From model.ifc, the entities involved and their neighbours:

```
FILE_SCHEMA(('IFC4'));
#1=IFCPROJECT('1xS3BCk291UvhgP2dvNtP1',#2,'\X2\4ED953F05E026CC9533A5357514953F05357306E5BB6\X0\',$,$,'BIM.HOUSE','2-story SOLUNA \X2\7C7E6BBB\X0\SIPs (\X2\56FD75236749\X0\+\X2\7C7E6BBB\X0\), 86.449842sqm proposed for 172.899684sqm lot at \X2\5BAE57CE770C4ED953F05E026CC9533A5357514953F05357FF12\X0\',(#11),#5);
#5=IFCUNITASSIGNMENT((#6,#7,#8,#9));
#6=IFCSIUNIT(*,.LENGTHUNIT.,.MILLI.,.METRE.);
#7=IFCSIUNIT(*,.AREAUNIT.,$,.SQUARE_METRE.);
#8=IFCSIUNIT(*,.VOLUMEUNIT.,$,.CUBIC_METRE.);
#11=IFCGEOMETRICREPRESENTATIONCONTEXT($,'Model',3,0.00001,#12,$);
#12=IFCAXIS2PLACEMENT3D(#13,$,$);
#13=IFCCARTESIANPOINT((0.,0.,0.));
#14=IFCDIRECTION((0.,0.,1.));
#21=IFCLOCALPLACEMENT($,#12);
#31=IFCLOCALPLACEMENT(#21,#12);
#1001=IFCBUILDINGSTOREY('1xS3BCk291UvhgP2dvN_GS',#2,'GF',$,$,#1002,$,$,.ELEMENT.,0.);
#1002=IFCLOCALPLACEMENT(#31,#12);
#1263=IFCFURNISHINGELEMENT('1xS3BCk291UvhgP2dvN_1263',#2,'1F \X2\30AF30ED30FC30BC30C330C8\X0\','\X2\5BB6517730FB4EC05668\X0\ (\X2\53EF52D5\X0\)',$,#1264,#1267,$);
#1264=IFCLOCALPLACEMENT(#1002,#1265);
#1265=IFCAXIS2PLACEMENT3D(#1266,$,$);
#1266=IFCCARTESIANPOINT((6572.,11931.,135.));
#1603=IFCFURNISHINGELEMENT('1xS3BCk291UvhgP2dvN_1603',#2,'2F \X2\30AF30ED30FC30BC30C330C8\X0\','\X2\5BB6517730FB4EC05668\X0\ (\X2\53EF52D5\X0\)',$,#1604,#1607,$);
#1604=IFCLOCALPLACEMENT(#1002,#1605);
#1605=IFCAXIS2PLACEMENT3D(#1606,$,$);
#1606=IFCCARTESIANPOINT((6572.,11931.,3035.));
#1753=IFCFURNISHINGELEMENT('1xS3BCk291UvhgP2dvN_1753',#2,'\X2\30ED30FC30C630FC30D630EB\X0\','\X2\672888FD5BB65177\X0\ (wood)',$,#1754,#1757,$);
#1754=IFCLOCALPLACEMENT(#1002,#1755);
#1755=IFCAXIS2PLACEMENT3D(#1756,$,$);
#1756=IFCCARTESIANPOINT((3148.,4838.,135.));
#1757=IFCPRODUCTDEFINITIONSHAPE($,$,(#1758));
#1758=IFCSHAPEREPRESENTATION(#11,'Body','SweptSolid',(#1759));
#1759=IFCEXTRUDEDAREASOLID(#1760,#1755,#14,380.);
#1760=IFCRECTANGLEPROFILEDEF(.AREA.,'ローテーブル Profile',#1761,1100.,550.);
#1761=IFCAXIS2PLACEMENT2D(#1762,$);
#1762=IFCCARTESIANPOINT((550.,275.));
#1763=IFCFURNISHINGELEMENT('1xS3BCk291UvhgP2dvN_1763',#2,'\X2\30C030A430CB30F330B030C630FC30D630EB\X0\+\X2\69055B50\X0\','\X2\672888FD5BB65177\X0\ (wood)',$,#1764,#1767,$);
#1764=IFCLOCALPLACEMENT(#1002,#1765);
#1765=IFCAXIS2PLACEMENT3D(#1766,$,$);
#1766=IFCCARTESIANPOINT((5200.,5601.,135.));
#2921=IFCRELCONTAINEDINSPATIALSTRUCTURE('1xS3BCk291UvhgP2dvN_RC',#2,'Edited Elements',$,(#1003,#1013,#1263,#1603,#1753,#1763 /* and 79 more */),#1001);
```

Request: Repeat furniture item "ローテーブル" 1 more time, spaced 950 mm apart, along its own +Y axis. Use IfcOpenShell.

```python
import ifcopenshell
import ifcopenshell.api.geometry
import ifcopenshell.api.root
import ifcopenshell.util.element
import ifcopenshell.util.placement
import ifcopenshell.util.unit

model = ifcopenshell.open("model.ifc")
unit_scale = ifcopenshell.util.unit.calculate_unit_scale(model)


def reuse_history(source, copy):
    """copy_class also copies each property set's owner history, people and application; keep the originals."""
    for rel in copy.IsDefinedBy:
        if rel.is_a("IfcRelDefinesByProperties") and (history := rel.RelatingPropertyDefinition.OwnerHistory):
            rel.RelatingPropertyDefinition.OwnerHistory = source.OwnerHistory
            ifcopenshell.util.element.remove_deep2(model, history)


source = model.by_guid("1xS3BCk291UvhgP2dvN_1753")
base = ifcopenshell.util.placement.get_local_placement(source.ObjectPlacement)
step = base[:3, 1] * 0.95 / unit_scale

for i in range(1, 2):
    copy = ifcopenshell.api.root.copy_class(model, product=source)
    copy.Representation = ifcopenshell.util.element.copy_deep(
        model, source.Representation, exclude=["IfcGeometricRepresentationContext", "IfcRepresentationMap"]
    )
    reuse_history(source, copy)
    matrix = base.copy()
    matrix[:3, 3] += i * step
    print("added at", matrix[:3, 3].round(3) + 0.0)
    ifcopenshell.api.geometry.edit_object_placement(model, product=copy, matrix=matrix, is_si=False)

model.write("model_v2.ifc")
```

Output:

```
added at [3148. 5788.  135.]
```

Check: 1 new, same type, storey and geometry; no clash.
